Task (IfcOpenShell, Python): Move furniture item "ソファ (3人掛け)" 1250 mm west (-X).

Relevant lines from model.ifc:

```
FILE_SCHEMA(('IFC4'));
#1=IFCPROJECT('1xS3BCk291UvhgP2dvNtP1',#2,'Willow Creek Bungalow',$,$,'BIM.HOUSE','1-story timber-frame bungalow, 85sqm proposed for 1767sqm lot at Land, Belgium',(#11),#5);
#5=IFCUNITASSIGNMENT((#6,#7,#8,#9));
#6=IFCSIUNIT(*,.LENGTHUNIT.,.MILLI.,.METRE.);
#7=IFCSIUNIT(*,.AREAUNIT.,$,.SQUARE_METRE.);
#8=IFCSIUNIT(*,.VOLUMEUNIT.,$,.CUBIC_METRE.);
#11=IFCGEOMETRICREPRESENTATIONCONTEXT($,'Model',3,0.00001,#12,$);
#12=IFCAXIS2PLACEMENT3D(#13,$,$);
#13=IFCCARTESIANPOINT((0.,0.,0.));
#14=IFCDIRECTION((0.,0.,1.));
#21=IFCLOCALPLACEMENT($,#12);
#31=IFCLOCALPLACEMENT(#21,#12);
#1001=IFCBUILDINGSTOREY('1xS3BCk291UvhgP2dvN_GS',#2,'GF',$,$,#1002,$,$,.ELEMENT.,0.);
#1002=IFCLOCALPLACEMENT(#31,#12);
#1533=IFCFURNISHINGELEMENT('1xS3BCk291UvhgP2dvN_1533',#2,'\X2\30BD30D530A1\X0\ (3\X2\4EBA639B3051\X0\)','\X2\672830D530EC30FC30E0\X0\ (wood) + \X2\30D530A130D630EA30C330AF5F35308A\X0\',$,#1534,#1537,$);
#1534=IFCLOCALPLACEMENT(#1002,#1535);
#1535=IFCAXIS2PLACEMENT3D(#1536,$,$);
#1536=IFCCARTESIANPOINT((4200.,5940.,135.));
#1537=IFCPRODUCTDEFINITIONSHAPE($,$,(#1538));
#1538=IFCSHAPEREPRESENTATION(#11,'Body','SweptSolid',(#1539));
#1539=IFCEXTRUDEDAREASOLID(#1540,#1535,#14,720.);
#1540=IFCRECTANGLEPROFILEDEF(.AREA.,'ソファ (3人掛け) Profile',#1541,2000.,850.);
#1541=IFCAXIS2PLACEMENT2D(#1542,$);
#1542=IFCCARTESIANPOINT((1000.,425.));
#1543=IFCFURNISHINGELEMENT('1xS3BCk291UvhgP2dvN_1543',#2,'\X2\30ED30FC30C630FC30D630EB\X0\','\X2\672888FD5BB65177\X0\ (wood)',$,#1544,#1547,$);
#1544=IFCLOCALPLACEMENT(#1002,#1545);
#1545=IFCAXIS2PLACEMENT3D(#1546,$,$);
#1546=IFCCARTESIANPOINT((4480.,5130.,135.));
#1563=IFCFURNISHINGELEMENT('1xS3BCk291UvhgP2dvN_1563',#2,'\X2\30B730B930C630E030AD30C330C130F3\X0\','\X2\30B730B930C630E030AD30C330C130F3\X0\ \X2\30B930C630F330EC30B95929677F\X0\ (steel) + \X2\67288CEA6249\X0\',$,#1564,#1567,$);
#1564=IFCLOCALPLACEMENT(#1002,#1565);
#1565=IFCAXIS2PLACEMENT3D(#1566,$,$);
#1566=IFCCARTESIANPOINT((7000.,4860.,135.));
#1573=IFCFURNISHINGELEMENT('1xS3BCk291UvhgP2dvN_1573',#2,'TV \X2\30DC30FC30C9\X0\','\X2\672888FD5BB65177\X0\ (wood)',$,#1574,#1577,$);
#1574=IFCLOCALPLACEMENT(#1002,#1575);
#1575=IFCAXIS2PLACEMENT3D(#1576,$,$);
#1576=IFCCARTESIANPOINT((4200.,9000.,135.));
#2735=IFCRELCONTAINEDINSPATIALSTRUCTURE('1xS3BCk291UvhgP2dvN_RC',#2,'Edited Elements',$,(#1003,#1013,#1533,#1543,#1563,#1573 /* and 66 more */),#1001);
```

```python
import ifcopenshell
import ifcopenshell.api.geometry
import ifcopenshell.util.placement
import ifcopenshell.util.unit

model = ifcopenshell.open("model.ifc")
unit_scale = ifcopenshell.util.unit.calculate_unit_scale(model)

item = model.by_guid("1xS3BCk291UvhgP2dvN_1533")
matrix = ifcopenshell.util.placement.get_local_placement(item.ObjectPlacement)
matrix[0, 3] -= 1.25 / unit_scale
ifcopenshell.api.geometry.edit_object_placement(model, product=item, matrix=matrix, is_si=False)

print(ifcopenshell.util.placement.get_local_placement(item.ObjectPlacement).round(3) + 0.0)

model.write("model-out.ifc")
```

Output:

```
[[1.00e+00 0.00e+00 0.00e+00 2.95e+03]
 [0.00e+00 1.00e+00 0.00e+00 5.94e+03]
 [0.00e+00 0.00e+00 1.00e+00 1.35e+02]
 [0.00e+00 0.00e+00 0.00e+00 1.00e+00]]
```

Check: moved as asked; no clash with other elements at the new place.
